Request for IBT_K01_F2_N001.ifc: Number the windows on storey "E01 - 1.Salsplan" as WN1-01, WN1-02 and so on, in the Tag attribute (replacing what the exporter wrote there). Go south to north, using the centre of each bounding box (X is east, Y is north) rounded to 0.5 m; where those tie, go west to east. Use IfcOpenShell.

First a look at what the model holds.

```python
import ifcopenshell
import ifcopenshell.util.element
import ifcopenshell.util.placement

model = ifcopenshell.open("IBT_K01_F2_N001.ifc")
print(model.schema)
storey = next(s for s in model.by_type("IfcBuildingStorey") if s.Name == "E01 - 1.Salsplan")
windows = [e for e in ifcopenshell.util.element.get_decomposition(storey) if e.is_a("IfcWindow")]
for e in sorted(windows, key=lambda e: e.id()):
    origin = ifcopenshell.util.placement.get_local_placement(e.ObjectPlacement)[:3, 3]
    print(e.id(), e.Tag, e.Name, origin.round(2) + 0.0, sep=" | ")
```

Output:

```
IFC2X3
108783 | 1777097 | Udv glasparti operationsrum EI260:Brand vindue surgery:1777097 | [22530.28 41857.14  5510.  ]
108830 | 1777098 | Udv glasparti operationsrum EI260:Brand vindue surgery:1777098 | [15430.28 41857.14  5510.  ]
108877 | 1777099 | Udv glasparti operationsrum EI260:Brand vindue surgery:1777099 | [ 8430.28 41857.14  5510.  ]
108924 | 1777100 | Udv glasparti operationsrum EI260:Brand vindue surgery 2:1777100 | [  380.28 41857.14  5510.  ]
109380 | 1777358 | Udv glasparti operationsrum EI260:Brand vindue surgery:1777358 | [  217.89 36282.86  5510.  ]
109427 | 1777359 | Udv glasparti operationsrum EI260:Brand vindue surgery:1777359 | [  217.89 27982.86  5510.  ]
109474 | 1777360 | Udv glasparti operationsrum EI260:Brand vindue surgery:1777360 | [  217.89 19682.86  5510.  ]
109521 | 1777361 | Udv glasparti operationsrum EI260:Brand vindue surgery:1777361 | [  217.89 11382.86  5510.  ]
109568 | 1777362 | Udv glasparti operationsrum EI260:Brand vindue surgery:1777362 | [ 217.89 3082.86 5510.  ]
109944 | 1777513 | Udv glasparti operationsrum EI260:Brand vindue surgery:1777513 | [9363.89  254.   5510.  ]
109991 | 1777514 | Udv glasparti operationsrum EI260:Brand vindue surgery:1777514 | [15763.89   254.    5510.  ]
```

```python
import ifcopenshell
import ifcopenshell.geom
import ifcopenshell.util.element
import ifcopenshell.util.shape

model = ifcopenshell.open("IBT_K01_F2_N001.ifc")
settings = ifcopenshell.geom.settings()
settings.set("use-world-coords", True)


def centre(element):
    shape = ifcopenshell.geom.create_shape(settings, element)
    return ifcopenshell.util.shape.get_bbox_centroid(shape.geometry)


storey = next(s for s in model.by_type("IfcBuildingStorey") if s.Name == "E01 - 1.Salsplan")
windows = [e for e in ifcopenshell.util.element.get_decomposition(storey) if e.is_a("IfcWindow")]

# Insertion points can sit at a corner or the storey origin, so sort by the geometry (in metres).
centres = {e: centre(e) for e in windows}
windows.sort(key=lambda e: (round(centres[e][1] / 0.5), centres[e][0]))

for i, e in enumerate(windows, start=1):
    number = f"WN1-{i:02d}"
    e.Tag = number
    print(e.id(), number)

model.write("IBT_K01_F2_N001_edited.ifc")
```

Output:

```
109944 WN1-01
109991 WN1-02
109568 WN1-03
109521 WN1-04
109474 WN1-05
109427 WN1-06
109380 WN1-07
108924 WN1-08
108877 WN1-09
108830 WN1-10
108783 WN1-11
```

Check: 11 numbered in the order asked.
